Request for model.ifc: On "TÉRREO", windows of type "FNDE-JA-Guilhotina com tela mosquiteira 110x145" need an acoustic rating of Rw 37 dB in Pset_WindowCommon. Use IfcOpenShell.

First a look at what the model holds.

```python
import ifcopenshell
import ifcopenshell.util.element

model = ifcopenshell.open("model.ifc")
print(model.schema)
storey = next(s for s in model.by_type("IfcBuildingStorey") if s.Name == "TÉRREO")
windows = [e for e in ifcopenshell.util.element.get_decomposition(storey) if e.is_a("IfcWindow")]
seen = {}
for e in windows:
    element_type = ifcopenshell.util.element.get_type(e)
    key = (element_type.Name if element_type != e and element_type else None, ifcopenshell.util.element.get_pset(e, "Pset_WindowCommon", "AcousticRating"))
    seen[key] = seen.get(key, 0) + 1
for (name, value), count in sorted(seen.items(), key=str):
    print(count, "x", name, "|", value)
```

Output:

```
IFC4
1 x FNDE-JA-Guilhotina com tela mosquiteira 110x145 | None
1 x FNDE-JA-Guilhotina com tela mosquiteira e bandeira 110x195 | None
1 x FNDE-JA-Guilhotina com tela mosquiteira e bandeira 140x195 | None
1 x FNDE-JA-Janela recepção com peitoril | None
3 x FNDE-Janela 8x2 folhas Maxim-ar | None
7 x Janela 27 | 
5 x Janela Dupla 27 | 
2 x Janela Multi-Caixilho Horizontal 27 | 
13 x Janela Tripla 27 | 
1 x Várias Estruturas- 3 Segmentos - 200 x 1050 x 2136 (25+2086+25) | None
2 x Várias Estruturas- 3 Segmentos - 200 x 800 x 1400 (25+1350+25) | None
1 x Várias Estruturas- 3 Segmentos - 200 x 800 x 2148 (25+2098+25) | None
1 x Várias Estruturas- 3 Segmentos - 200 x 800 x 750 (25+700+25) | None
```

```python
import ifcopenshell
import ifcopenshell.api.pset
import ifcopenshell.util.element

model = ifcopenshell.open("model.ifc")

storey = next(s for s in model.by_type("IfcBuildingStorey") if s.Name == "TÉRREO")
windows = [e for e in ifcopenshell.util.element.get_decomposition(storey) if e.is_a("IfcWindow")]

count = 0
for e in windows:
    element_type = ifcopenshell.util.element.get_type(e)
    if element_type in (None, e) or element_type.Name != "FNDE-JA-Guilhotina com tela mosquiteira 110x145":
        continue
    # add_pset returns the element's existing set when there is one.
    pset = ifcopenshell.api.pset.add_pset(model, product=e, name="Pset_WindowCommon")
    ifcopenshell.api.pset.edit_pset(model, pset=pset, properties={"AcousticRating": "Rw 37 dB"})
    count += 1

print(count, "windows updated")

model.write("model_updated.ifc")
```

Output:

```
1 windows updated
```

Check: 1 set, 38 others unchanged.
